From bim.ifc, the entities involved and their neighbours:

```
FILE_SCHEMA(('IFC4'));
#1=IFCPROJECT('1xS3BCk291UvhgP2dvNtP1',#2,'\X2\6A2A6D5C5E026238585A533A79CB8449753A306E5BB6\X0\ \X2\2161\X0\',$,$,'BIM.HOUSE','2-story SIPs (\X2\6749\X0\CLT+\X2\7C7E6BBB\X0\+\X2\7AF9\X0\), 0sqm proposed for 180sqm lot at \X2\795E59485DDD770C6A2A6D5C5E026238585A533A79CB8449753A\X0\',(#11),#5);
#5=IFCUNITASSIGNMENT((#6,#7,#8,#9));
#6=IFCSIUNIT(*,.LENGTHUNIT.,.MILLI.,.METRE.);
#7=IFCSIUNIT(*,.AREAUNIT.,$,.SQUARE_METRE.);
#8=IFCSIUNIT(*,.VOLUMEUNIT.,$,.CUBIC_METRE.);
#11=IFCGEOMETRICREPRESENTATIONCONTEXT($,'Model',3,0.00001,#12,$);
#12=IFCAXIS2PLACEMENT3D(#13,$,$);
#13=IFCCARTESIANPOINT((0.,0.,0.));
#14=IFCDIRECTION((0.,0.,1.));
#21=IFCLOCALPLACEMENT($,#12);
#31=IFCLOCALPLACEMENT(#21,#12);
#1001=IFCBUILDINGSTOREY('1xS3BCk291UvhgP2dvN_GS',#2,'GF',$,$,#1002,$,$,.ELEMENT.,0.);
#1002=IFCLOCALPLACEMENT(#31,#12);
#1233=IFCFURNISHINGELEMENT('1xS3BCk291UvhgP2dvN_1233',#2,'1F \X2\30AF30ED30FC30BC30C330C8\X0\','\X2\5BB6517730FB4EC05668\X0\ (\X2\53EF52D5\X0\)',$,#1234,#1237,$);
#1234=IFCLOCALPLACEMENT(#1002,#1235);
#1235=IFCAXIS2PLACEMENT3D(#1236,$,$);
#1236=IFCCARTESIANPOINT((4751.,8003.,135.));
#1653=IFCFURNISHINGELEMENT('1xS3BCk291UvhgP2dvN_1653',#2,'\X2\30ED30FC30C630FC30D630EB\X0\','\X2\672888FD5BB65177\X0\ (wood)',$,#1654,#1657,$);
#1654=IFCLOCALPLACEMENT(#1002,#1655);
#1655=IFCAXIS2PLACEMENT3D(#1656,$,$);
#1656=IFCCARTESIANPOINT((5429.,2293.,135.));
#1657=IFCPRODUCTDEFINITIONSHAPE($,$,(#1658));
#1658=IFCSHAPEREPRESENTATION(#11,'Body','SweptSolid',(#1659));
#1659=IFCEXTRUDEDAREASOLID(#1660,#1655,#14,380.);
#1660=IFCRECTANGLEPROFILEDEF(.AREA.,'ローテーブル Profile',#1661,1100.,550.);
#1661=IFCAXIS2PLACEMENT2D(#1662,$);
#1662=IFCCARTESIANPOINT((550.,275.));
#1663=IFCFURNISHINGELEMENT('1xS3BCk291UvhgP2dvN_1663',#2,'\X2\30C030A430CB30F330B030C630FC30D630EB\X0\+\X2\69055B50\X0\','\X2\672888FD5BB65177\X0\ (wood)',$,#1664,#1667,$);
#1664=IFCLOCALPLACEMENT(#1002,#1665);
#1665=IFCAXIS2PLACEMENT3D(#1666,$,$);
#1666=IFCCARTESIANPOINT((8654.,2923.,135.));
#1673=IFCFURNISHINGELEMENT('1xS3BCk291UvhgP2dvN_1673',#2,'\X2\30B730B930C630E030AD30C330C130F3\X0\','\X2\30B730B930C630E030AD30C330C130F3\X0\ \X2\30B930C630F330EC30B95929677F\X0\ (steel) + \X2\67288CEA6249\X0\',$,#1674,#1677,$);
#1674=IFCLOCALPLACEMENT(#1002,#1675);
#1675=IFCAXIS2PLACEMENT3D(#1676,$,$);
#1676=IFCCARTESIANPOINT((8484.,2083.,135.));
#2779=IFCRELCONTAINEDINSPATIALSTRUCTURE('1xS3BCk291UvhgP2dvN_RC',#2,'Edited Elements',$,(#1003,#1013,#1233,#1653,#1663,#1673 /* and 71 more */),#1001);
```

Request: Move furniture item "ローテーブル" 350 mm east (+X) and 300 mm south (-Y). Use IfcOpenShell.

```python
import ifcopenshell
import ifcopenshell.api.geometry
import ifcopenshell.util.placement
import ifcopenshell.util.unit

model = ifcopenshell.open("bim.ifc")
unit_scale = ifcopenshell.util.unit.calculate_unit_scale(model)

item = model.by_id(1653)
matrix = ifcopenshell.util.placement.get_local_placement(item.ObjectPlacement)
matrix[0, 3] += 0.35 / unit_scale
matrix[1, 3] -= 0.3 / unit_scale
ifcopenshell.api.geometry.edit_object_placement(model, product=item, matrix=matrix, is_si=False)

print(ifcopenshell.util.placement.get_local_placement(item.ObjectPlacement).round(3) + 0.0)

model.write("bim_v2.ifc")
```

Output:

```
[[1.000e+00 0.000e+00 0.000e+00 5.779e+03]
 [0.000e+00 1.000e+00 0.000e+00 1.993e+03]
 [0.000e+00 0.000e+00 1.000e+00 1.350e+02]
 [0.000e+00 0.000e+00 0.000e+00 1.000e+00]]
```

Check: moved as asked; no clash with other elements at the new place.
